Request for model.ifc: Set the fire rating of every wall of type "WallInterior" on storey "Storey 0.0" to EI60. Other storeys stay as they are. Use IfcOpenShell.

First a look at what the model holds.

```python
import ifcopenshell
import ifcopenshell.util.element

model = ifcopenshell.open("model.ifc")
print(model.schema)
storey = next(s for s in model.by_type("IfcBuildingStorey") if s.Name == "Storey 0.0")
walls = [e for e in ifcopenshell.util.element.get_decomposition(storey) if e.is_a("IfcWall")]
seen = {}
for e in walls:
    element_type = ifcopenshell.util.element.get_type(e)
    key = (element_type.Name if element_type != e and element_type else None, ifcopenshell.util.element.get_pset(e, "Pset_WallCommon", "FireRating"))
    seen[key] = seen.get(key, 0) + 1
for (name, value), count in sorted(seen.items(), key=str):
    print(count, "x", name, "|", value)
```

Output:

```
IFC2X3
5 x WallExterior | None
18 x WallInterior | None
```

```python
import ifcopenshell
import ifcopenshell.api.pset
import ifcopenshell.util.element

model = ifcopenshell.open("model.ifc")

storey = next(s for s in model.by_type("IfcBuildingStorey") if s.Name == "Storey 0.0")
walls = [e for e in ifcopenshell.util.element.get_decomposition(storey) if e.is_a("IfcWall")]

count = 0
for e in walls:
    element_type = ifcopenshell.util.element.get_type(e)
    if element_type in (None, e) or element_type.Name != "WallInterior":
        continue
    # add_pset returns the element's existing set when there is one.
    pset = ifcopenshell.api.pset.add_pset(model, product=e, name="Pset_WallCommon")
    ifcopenshell.api.pset.edit_pset(model, pset=pset, properties={"FireRating": "EI60"})
    count += 1

print(count, "walls updated")

model.write("model_updated.ifc")
```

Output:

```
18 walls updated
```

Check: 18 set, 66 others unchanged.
